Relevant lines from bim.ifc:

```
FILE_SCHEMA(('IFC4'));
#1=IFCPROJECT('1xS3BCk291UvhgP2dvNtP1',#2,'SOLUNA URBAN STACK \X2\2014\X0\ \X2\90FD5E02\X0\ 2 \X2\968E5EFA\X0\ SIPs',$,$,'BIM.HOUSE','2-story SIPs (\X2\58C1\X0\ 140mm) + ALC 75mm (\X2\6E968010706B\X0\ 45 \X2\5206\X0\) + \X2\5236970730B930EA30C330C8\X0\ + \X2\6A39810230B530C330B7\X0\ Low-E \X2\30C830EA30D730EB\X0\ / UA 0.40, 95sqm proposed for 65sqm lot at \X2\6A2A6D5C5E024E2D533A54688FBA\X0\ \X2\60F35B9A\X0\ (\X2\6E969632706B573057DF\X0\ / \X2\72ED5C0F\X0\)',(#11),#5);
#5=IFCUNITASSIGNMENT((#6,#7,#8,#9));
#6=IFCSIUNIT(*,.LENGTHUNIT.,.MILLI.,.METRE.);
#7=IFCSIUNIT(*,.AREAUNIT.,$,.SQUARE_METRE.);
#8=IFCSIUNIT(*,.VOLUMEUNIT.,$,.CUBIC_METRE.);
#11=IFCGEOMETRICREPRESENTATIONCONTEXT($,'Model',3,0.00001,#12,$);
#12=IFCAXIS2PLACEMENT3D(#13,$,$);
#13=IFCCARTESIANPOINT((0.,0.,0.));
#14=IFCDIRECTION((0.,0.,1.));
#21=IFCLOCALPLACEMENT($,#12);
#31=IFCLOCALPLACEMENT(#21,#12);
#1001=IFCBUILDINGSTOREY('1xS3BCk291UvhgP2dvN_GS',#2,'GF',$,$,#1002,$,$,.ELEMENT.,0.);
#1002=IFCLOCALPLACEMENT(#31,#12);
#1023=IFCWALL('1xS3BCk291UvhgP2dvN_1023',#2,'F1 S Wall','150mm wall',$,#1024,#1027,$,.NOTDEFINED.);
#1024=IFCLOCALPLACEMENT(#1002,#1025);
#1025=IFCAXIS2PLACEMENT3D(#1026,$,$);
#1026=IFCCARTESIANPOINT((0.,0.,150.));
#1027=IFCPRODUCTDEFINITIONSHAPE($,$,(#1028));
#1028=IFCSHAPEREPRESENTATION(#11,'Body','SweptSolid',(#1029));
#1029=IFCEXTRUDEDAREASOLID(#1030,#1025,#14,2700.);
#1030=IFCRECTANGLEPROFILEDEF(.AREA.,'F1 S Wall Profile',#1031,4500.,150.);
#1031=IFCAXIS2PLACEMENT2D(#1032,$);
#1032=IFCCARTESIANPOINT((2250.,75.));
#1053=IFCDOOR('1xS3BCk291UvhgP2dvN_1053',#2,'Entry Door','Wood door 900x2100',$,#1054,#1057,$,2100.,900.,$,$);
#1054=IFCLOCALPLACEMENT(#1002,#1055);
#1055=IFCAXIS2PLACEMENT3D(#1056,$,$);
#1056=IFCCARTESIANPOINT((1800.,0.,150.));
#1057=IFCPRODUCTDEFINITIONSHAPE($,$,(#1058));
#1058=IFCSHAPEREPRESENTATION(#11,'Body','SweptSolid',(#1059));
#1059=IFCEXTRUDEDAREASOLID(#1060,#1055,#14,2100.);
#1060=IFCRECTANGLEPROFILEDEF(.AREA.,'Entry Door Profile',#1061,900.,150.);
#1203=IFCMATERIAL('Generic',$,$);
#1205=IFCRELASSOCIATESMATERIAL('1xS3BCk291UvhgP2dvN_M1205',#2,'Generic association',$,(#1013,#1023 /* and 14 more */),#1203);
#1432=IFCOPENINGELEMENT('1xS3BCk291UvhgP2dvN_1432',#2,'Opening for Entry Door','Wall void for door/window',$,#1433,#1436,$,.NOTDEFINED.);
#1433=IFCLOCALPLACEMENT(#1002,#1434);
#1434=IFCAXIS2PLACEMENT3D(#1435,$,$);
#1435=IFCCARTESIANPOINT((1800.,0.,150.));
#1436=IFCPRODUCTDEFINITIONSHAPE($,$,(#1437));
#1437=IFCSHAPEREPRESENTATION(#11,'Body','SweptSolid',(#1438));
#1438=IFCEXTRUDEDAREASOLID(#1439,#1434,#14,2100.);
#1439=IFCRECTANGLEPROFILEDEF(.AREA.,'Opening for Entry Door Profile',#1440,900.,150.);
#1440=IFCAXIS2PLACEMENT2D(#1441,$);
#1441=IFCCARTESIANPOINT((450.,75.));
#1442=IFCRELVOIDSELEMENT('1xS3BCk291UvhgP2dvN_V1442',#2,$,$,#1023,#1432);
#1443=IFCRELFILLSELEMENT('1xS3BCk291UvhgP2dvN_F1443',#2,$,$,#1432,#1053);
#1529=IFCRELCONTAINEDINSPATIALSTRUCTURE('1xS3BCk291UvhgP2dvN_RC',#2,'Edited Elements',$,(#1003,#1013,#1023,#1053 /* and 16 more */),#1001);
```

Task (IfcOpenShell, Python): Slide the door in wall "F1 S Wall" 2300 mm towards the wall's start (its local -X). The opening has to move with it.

```python
import ifcopenshell
import ifcopenshell.api.geometry
import ifcopenshell.util.placement
import ifcopenshell.util.unit

model = ifcopenshell.open("bim.ifc")
unit_scale = ifcopenshell.util.unit.calculate_unit_scale(model)

door = model.by_guid("1xS3BCk291UvhgP2dvN_1053")
opening = door.FillsVoids[0].RelatingOpeningElement
wall = opening.VoidsElements[0].RelatingBuildingElement

wall_matrix = ifcopenshell.util.placement.get_local_placement(wall.ObjectPlacement)
shift = wall_matrix[:3, 0] * -2.3 / unit_scale
before = ifcopenshell.util.placement.get_local_placement(door.ObjectPlacement)[:3, 3].copy()

# The door is not placed relative to its opening, so move both.
for product in (opening, door):
    matrix = ifcopenshell.util.placement.get_local_placement(product.ObjectPlacement)
    matrix[:3, 3] += shift
    ifcopenshell.api.geometry.edit_object_placement(model, product=product, matrix=matrix, is_si=False)

after = ifcopenshell.util.placement.get_local_placement(door.ObjectPlacement)[:3, 3]
print("door moved by", (after - before).round(3) + 0.0)

model.write("bim_updated.ifc")
```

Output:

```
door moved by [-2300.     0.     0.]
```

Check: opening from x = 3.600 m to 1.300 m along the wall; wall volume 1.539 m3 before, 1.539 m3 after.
